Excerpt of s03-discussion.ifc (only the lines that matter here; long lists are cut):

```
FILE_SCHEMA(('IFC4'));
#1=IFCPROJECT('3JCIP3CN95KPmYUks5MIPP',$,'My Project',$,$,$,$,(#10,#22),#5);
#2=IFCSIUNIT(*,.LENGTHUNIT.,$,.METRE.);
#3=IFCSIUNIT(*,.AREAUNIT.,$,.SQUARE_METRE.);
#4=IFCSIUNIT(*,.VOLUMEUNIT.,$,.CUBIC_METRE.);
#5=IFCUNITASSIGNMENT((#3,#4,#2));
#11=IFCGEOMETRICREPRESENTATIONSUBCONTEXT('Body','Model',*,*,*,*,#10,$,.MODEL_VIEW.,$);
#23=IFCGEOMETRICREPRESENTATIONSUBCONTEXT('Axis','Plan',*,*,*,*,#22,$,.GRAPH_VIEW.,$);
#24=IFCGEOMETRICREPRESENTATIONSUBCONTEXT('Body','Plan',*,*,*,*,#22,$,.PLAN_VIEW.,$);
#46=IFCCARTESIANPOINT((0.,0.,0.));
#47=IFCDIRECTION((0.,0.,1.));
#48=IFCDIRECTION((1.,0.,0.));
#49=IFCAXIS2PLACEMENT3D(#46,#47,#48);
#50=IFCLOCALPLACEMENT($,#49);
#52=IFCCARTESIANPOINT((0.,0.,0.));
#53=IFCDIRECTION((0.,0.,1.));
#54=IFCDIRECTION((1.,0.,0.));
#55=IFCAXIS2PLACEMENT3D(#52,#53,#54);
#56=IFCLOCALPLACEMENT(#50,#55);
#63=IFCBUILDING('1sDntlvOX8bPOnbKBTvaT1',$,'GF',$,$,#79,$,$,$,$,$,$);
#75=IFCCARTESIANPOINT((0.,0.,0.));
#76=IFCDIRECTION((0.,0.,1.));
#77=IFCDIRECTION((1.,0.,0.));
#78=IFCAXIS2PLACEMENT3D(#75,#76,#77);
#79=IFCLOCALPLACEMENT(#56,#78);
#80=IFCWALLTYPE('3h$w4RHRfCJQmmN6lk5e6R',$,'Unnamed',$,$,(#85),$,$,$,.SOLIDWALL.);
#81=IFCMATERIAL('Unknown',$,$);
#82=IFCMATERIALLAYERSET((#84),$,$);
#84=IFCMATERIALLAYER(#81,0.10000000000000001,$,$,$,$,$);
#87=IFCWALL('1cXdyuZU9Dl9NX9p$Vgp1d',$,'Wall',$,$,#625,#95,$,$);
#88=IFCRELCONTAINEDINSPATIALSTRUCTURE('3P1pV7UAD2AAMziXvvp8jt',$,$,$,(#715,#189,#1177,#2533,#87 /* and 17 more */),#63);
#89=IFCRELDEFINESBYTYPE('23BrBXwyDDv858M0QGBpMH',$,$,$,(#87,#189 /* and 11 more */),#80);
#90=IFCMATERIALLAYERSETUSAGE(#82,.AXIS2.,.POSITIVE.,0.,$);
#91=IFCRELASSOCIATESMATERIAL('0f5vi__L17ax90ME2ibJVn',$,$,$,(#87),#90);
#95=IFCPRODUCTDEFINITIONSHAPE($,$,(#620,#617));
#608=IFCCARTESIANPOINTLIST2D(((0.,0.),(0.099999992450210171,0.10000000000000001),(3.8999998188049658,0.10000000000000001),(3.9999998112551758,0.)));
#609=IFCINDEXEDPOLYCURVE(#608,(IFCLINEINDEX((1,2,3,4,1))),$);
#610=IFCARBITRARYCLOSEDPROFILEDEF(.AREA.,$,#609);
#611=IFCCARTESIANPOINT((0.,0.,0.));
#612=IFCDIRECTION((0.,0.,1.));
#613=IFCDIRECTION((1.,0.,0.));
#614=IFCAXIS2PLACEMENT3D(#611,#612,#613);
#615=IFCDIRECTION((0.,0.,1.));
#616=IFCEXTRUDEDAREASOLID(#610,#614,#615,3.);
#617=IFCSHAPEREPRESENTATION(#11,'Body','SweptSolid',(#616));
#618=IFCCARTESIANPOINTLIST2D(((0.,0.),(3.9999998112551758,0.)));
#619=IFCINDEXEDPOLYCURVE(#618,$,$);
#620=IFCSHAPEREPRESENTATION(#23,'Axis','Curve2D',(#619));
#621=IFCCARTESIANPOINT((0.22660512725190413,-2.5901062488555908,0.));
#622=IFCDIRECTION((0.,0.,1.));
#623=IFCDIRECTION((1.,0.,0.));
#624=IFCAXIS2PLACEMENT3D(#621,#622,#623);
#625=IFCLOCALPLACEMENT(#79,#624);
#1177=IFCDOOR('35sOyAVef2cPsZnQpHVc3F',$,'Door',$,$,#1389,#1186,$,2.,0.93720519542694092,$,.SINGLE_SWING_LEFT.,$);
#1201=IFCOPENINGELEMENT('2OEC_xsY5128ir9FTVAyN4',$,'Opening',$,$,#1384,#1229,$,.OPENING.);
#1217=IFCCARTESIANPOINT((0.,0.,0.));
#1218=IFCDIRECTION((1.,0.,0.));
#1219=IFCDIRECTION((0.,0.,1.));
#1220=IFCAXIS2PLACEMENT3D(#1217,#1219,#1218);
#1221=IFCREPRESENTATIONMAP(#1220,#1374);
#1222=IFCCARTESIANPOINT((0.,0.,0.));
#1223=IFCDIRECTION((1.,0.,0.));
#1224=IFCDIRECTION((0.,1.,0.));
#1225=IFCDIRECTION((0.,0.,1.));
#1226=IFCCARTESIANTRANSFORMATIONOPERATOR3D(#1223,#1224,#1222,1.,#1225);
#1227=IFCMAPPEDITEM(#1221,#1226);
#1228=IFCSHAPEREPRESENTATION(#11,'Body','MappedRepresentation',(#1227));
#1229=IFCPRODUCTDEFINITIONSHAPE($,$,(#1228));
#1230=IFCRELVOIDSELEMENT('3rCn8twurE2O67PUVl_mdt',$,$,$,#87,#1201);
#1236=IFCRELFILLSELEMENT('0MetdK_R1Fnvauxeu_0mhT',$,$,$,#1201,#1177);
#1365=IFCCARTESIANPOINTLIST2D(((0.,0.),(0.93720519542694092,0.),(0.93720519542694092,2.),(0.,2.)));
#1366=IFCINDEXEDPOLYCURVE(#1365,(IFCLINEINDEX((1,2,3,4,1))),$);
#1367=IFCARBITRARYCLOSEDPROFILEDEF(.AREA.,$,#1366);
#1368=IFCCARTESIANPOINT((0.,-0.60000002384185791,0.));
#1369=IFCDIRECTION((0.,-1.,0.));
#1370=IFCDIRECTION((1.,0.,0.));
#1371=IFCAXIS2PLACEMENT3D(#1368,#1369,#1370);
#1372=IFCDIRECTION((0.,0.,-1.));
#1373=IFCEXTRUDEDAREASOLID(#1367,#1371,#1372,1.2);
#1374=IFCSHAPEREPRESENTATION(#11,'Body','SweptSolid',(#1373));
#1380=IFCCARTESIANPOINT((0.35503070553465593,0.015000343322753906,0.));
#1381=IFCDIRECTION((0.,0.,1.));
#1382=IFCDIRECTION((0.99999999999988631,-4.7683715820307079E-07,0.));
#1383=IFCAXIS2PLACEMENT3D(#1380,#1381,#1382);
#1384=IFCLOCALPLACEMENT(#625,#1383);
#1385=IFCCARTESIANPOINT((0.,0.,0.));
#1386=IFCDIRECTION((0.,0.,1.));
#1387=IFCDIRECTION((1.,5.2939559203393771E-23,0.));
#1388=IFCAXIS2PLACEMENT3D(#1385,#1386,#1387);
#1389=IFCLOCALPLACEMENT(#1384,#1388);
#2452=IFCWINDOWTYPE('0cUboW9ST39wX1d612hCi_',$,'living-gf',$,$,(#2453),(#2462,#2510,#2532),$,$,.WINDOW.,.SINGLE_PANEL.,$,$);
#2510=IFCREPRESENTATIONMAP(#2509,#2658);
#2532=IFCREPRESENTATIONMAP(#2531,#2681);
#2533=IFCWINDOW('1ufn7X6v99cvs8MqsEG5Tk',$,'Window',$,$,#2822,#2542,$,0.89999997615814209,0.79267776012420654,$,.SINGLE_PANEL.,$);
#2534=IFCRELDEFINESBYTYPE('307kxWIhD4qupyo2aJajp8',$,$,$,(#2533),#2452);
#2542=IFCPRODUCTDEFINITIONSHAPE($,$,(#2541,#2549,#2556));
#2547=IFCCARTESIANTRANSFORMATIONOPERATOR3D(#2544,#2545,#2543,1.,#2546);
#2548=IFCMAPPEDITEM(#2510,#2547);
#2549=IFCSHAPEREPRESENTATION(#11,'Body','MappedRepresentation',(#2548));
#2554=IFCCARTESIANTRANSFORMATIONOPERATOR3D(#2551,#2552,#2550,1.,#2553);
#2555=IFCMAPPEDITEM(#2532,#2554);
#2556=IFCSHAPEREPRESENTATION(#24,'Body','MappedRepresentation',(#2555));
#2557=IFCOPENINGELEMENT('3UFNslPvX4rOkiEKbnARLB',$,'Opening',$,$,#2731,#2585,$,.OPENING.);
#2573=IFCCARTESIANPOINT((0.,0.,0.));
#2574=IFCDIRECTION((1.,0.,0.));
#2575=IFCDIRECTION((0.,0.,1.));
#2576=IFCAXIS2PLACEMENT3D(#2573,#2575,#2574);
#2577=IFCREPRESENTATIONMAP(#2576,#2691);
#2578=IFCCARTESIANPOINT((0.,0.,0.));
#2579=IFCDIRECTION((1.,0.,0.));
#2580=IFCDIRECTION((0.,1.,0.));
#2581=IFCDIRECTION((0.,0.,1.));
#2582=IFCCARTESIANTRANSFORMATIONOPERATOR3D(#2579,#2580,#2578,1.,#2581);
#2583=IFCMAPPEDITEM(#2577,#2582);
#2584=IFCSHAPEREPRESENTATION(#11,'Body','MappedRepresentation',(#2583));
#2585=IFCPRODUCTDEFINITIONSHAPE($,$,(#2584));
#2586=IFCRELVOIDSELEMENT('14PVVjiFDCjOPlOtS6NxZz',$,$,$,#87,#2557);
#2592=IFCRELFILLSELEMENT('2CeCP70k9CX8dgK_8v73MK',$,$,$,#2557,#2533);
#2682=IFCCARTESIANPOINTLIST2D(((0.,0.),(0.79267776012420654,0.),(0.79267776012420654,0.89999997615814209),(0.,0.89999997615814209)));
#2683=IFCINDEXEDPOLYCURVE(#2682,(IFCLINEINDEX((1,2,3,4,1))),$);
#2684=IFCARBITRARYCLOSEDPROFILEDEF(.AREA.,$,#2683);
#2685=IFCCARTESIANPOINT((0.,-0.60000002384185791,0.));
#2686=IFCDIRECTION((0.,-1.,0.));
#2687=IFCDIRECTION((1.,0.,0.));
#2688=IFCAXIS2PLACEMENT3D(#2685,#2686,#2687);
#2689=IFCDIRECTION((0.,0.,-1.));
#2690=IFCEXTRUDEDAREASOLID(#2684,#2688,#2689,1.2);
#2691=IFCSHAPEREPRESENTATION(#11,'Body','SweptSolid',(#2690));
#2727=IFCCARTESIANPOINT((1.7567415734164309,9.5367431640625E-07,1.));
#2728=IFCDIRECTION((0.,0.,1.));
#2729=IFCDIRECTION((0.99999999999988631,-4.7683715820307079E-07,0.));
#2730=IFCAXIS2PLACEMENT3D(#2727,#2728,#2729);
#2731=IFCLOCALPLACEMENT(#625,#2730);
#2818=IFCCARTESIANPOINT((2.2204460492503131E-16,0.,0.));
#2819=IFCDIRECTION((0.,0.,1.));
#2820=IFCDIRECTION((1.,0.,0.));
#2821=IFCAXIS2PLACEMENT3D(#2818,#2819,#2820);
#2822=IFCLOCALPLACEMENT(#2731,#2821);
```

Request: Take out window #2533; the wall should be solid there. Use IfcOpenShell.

```python
import ifcopenshell
import ifcopenshell.api.feature
import ifcopenshell.api.root
import ifcopenshell.geom
import ifcopenshell.util.shape

model = ifcopenshell.open("s03-discussion.ifc")
settings = ifcopenshell.geom.settings()


def volume(element):
    """Net volume in cubic metres, openings subtracted."""
    shape = ifcopenshell.geom.create_shape(settings, element)
    return ifcopenshell.util.shape.get_volume(shape.geometry)


window = model.by_guid("1ufn7X6v99cvs8MqsEG5Tk")
opening = window.FillsVoids[0].RelatingOpeningElement
wall = opening.VoidsElements[0].RelatingBuildingElement
before = volume(wall)

ifcopenshell.api.root.remove_product(model, product=window)
ifcopenshell.api.feature.remove_feature(model, feature=opening)

after = volume(wall)

print(f"wall volume {before:.3f} -> {after:.3f} m3")

model.write("s03-discussion_v2.ifc")
```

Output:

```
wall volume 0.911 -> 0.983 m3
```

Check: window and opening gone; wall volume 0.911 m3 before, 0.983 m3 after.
